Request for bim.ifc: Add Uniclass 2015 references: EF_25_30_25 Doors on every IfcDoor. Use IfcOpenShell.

First a look at what the model holds.

```python
import ifcopenshell

model = ifcopenshell.open("bim.ifc")
print(model.schema)
print("classifications:", [c.Name for c in model.by_type("IfcClassification")])
for ifc_class in ("IfcDoor", "IfcRoof", "IfcStair", "IfcWall", "IfcWindow"):
    print(ifc_class, len(model.by_type(ifc_class)))
```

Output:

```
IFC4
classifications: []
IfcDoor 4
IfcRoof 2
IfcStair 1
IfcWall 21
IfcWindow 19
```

```python
import ifcopenshell
import ifcopenshell.api.classification

model = ifcopenshell.open("bim.ifc")

system = ifcopenshell.api.classification.add_classification(model, classification="Uniclass 2015")

codes = {
    "IfcDoor": ("EF_25_30_25", "Doors"),
}
for ifc_class, (code, name) in codes.items():
    products = model.by_type(ifc_class)
    ifcopenshell.api.classification.add_reference(
        model, products=products, classification=system, identification=code, name=name
    )
    print(code, len(products))

model.write("bim-out.ifc")
```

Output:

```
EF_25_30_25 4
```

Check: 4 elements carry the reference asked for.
